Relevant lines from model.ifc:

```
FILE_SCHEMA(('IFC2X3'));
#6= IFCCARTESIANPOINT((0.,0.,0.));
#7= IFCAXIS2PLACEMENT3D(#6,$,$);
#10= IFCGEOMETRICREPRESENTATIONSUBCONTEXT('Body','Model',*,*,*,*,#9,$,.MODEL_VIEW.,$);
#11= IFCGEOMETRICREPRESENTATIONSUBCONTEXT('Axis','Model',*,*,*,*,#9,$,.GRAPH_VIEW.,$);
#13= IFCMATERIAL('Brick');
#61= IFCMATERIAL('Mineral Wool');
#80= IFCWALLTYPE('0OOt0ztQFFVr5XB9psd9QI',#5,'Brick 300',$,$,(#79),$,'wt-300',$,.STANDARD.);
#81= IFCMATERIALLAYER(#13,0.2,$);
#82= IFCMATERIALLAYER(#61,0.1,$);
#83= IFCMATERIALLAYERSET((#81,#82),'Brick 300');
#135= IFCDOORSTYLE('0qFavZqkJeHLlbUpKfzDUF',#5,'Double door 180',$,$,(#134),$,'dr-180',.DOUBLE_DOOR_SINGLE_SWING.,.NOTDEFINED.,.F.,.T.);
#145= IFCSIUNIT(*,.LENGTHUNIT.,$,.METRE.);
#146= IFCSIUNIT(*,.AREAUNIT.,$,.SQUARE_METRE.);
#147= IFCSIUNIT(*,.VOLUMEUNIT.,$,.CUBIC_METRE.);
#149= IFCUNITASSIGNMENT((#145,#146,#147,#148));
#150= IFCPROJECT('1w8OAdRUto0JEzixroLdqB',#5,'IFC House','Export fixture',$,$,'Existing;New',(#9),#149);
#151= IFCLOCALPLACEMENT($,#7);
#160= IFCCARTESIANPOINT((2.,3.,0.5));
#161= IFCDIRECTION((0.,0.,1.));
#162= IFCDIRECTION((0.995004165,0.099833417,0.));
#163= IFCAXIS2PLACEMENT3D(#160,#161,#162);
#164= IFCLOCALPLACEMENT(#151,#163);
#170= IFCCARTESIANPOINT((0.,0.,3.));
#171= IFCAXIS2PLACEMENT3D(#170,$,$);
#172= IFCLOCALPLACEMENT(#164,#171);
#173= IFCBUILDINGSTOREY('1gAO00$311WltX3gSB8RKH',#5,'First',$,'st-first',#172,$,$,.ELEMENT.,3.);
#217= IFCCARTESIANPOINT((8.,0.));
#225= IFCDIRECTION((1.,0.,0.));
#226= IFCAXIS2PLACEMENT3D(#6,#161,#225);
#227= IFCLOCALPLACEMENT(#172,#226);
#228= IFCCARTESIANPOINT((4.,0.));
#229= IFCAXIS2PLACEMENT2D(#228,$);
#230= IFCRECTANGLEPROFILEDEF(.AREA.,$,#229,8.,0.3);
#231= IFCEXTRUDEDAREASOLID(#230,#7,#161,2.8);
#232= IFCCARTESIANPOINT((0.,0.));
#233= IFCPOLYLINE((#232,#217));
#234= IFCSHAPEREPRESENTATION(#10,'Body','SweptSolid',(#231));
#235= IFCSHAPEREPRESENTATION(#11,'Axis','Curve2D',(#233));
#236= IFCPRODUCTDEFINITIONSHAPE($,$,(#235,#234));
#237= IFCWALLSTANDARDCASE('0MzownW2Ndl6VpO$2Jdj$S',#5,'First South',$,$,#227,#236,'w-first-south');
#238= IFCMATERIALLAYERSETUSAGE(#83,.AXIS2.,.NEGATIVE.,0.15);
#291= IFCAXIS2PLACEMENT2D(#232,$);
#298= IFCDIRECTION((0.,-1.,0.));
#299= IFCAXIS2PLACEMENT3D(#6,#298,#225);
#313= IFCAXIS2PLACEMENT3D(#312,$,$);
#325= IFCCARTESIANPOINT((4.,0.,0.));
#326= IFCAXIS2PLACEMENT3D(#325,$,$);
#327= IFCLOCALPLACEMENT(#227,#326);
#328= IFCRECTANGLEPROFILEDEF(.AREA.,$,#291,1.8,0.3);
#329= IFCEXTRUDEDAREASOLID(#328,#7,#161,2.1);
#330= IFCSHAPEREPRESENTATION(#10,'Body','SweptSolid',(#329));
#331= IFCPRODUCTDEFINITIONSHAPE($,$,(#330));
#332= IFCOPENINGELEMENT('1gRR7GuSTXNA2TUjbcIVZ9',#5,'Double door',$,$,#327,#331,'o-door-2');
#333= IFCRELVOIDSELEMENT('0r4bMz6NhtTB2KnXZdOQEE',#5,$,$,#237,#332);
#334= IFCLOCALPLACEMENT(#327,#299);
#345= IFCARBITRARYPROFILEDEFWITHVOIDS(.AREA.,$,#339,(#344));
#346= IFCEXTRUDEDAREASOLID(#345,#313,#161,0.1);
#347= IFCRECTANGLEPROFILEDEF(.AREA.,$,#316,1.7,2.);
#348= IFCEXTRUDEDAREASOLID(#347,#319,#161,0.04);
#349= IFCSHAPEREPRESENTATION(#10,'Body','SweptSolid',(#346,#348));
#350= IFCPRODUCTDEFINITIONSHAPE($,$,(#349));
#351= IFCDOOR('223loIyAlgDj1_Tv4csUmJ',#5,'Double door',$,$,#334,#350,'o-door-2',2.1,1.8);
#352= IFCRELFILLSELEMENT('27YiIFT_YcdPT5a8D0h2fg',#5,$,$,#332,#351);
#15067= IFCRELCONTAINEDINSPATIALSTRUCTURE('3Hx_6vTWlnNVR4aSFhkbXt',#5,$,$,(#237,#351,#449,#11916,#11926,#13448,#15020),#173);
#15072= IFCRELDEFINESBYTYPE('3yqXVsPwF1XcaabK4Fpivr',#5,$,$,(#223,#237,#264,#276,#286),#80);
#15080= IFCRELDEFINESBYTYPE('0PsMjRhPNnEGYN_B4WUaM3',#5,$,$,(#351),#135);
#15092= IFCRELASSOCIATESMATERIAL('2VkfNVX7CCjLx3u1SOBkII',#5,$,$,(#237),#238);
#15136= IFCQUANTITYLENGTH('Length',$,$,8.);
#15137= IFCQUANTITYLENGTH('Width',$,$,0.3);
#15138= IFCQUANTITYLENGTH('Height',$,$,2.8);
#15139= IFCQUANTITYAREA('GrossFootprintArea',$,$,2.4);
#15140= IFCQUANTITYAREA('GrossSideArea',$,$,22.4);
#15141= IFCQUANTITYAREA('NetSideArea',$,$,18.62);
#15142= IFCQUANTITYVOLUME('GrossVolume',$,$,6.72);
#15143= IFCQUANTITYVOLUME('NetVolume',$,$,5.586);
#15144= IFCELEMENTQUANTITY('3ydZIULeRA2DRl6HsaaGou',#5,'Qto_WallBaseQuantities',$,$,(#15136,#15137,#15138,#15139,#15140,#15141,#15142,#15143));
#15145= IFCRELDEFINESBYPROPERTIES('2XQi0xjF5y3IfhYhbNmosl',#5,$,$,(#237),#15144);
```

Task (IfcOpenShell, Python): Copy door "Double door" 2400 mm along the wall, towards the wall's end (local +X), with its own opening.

```python
import ifcopenshell
import ifcopenshell.api.feature
import ifcopenshell.api.geometry
import ifcopenshell.api.pset
import ifcopenshell.api.root
import ifcopenshell.geom
import ifcopenshell.util.element
import ifcopenshell.util.placement
import ifcopenshell.util.shape
import ifcopenshell.util.unit

model = ifcopenshell.open("model.ifc")
unit_scale = ifcopenshell.util.unit.calculate_unit_scale(model)
area_scale = ifcopenshell.util.unit.calculate_unit_scale(model, "AREAUNIT")
volume_scale = ifcopenshell.util.unit.calculate_unit_scale(model, "VOLUMEUNIT")
settings = ifcopenshell.geom.settings()


def volume(element):
    """Net volume in cubic metres, openings subtracted."""
    shape = ifcopenshell.geom.create_shape(settings, element)
    return ifcopenshell.util.shape.get_volume(shape.geometry)


def reuse_history(source, copy):
    """copy_class also copies each property set's owner history, people and application; keep the originals."""
    for rel in copy.IsDefinedBy:
        if rel.is_a("IfcRelDefinesByProperties") and (history := rel.RelatingPropertyDefinition.OwnerHistory):
            rel.RelatingPropertyDefinition.OwnerHistory = source.OwnerHistory
            ifcopenshell.util.element.remove_deep2(model, history)


door = model.by_id(351)
opening = door.FillsVoids[0].RelatingOpeningElement
wall = opening.VoidsElements[0].RelatingBuildingElement
before = volume(wall)
shift = ifcopenshell.util.placement.get_local_placement(wall.ObjectPlacement)[:3, 0] * 2.4 / unit_scale

# copy_class copies the void relationship, type, container and properties, but no geometry.
new_opening = ifcopenshell.api.root.copy_class(model, product=opening)
new_opening.Representation = ifcopenshell.util.element.copy_deep(
    model, opening.Representation, exclude=["IfcGeometricRepresentationContext", "IfcRepresentationMap"]
)
new_opening.Tag = None
new_door = ifcopenshell.api.root.copy_class(model, product=door)
new_door.Representation = ifcopenshell.util.element.copy_deep(
    model, door.Representation, exclude=["IfcGeometricRepresentationContext", "IfcRepresentationMap"]
)
new_door.Tag = None
reuse_history(door, new_door)
fills = ifcopenshell.api.feature.add_filling(model, opening=new_opening, element=new_door)
fills.OwnerHistory = new_door.OwnerHistory  # required in IFC2X3

for old, new in ((opening, new_opening), (door, new_door)):
    matrix = ifcopenshell.util.placement.get_local_placement(old.ObjectPlacement)
    matrix[:3, 3] += shift
    ifcopenshell.api.geometry.edit_object_placement(model, product=new, matrix=matrix, is_si=False)

after = volume(wall)
thickness = 0.3  # wall thickness in metres

# Update the wall's stored quantities.
qto = model.by_id(ifcopenshell.util.element.get_pset(wall, "Qto_WallBaseQuantities", should_inherit=False)["id"])
ifcopenshell.api.pset.edit_qto(model, qto=qto, properties={
    "NetSideArea": after / thickness / area_scale,
    "NetVolume": after / volume_scale,
})

print(f"wall volume {before:.3f} -> {after:.3f} m3")

model.write("model_updated.ifc")
```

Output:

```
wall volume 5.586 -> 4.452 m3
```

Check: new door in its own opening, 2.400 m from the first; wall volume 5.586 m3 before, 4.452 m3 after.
